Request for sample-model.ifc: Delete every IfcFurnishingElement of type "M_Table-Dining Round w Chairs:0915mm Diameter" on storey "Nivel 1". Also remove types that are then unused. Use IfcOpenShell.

First a look at what the model holds.

```python
import ifcopenshell
import ifcopenshell.util.element

model = ifcopenshell.open("sample-model.ifc")
print(model.schema)
storey = next(s for s in model.by_type("IfcBuildingStorey") if s.Name == "Nivel 1")
furniture = [e for e in ifcopenshell.util.element.get_decomposition(storey) if e.is_a("IfcFurnishingElement")]
seen = {}
for e in furniture:
    element_type = ifcopenshell.util.element.get_type(e)
    name = element_type.Name if element_type not in (None, e) else None
    seen[name] = seen.get(name, 0) + 1
for name, count in sorted(seen.items(), key=str):
    print(count, "x", name)
```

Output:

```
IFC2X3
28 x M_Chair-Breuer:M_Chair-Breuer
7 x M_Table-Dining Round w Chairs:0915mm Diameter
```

```python
import ifcopenshell
import ifcopenshell.api.root
import ifcopenshell.util.element

model = ifcopenshell.open("sample-model.ifc")

storey = next(s for s in model.by_type("IfcBuildingStorey") if s.Name == "Nivel 1")
furniture = [e for e in ifcopenshell.util.element.get_decomposition(storey) if e.is_a("IfcFurnishingElement")]
targets = [e for e in furniture if (t := ifcopenshell.util.element.get_type(e)) not in (None, e) and t.Name == "M_Table-Dining Round w Chairs:0915mm Diameter"]
types = {ifcopenshell.util.element.get_type(e) for e in targets} - {None, *targets}

for e in targets:
    ifcopenshell.api.root.remove_product(model, product=e)
print(len(targets), "removed")

unused = [t for t in types if not ifcopenshell.util.element.get_types(t)]
for t in unused:
    ifcopenshell.api.root.remove_product(model, product=t)
print(len(unused), "unused types removed")

model.write("sample-model_rev.ifc")
```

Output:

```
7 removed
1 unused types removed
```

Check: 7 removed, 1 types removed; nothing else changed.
